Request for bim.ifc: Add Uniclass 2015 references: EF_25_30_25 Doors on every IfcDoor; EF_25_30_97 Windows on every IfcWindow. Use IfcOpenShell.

First a look at what the model holds.

```python
import ifcopenshell

model = ifcopenshell.open("bim.ifc")
print(model.schema)
print("classifications:", [c.Name for c in model.by_type("IfcClassification")])
for ifc_class in ("IfcDoor", "IfcRoof", "IfcStair", "IfcWall", "IfcWindow"):
    print(ifc_class, len(model.by_type(ifc_class)))
```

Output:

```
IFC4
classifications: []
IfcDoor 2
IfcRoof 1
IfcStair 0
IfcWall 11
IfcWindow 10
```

```python
import ifcopenshell
import ifcopenshell.api.classification

model = ifcopenshell.open("bim.ifc")

system = ifcopenshell.api.classification.add_classification(model, classification="Uniclass 2015")

codes = {
    "IfcDoor": ("EF_25_30_25", "Doors"),
    "IfcWindow": ("EF_25_30_97", "Windows"),
}
for ifc_class, (code, name) in codes.items():
    products = model.by_type(ifc_class)
    ifcopenshell.api.classification.add_reference(
        model, products=products, classification=system, identification=code, name=name
    )
    print(code, len(products))

model.write("bim_edited.ifc")
```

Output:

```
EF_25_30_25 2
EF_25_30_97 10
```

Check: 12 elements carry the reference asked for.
